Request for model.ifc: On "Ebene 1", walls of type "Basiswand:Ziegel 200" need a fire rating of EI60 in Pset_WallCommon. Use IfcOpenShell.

First a look at what the model holds.

```python
import ifcopenshell
import ifcopenshell.util.element

model = ifcopenshell.open("model.ifc")
print(model.schema)
storey = next(s for s in model.by_type("IfcBuildingStorey") if s.Name == "Ebene 1")
walls = [e for e in ifcopenshell.util.element.get_decomposition(storey) if e.is_a("IfcWall")]
seen = {}
for e in walls:
    element_type = ifcopenshell.util.element.get_type(e)
    key = (element_type.Name if element_type != e and element_type else None, ifcopenshell.util.element.get_pset(e, "Pset_WallCommon", "FireRating"))
    seen[key] = seen.get(key, 0) + 1
for (name, value), count in sorted(seen.items(), key=str):
    print(count, "x", name, "|", value)
```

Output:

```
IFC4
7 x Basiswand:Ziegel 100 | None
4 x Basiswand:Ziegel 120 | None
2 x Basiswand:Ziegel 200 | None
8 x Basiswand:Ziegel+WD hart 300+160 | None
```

```python
import ifcopenshell
import ifcopenshell.api.pset
import ifcopenshell.util.element

model = ifcopenshell.open("model.ifc")

storey = next(s for s in model.by_type("IfcBuildingStorey") if s.Name == "Ebene 1")
walls = [e for e in ifcopenshell.util.element.get_decomposition(storey) if e.is_a("IfcWall")]

count = 0
for e in walls:
    element_type = ifcopenshell.util.element.get_type(e)
    if element_type in (None, e) or element_type.Name != "Basiswand:Ziegel 200":
        continue
    # add_pset returns the element's existing set when there is one.
    pset = ifcopenshell.api.pset.add_pset(model, product=e, name="Pset_WallCommon")
    ifcopenshell.api.pset.edit_pset(model, pset=pset, properties={"FireRating": "EI60"})
    count += 1

print(count, "walls updated")

model.write("model_rev.ifc")
```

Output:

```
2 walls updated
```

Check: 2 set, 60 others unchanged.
